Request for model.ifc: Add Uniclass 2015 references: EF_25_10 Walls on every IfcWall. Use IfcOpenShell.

First a look at what the model holds.

```python
import ifcopenshell

model = ifcopenshell.open("model.ifc")
print(model.schema)
print("classifications:", [c.Name for c in model.by_type("IfcClassification")])
for ifc_class in ("IfcDoor", "IfcRoof", "IfcStair", "IfcWall", "IfcWindow"):
    print(ifc_class, len(model.by_type(ifc_class)))
```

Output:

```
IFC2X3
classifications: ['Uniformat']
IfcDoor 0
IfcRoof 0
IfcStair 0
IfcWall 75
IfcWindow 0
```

```python
import ifcopenshell
import ifcopenshell.api.classification

model = ifcopenshell.open("model.ifc")

# IFC2X3 requires Source and Edition and has no link from the project to the system.
system = model.create_entity("IfcClassification", Source="NBS", Edition="2015", Name="Uniclass 2015")

codes = {
    "IfcWall": ("EF_25_10", "Walls"),
}
for ifc_class, (code, name) in codes.items():
    products = model.by_type(ifc_class)
    ifcopenshell.api.classification.add_reference(
        model, products=products, classification=system, identification=code, name=name
    )
    print(code, len(products))

model.write("model-out.ifc")
```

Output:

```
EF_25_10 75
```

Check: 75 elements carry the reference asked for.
